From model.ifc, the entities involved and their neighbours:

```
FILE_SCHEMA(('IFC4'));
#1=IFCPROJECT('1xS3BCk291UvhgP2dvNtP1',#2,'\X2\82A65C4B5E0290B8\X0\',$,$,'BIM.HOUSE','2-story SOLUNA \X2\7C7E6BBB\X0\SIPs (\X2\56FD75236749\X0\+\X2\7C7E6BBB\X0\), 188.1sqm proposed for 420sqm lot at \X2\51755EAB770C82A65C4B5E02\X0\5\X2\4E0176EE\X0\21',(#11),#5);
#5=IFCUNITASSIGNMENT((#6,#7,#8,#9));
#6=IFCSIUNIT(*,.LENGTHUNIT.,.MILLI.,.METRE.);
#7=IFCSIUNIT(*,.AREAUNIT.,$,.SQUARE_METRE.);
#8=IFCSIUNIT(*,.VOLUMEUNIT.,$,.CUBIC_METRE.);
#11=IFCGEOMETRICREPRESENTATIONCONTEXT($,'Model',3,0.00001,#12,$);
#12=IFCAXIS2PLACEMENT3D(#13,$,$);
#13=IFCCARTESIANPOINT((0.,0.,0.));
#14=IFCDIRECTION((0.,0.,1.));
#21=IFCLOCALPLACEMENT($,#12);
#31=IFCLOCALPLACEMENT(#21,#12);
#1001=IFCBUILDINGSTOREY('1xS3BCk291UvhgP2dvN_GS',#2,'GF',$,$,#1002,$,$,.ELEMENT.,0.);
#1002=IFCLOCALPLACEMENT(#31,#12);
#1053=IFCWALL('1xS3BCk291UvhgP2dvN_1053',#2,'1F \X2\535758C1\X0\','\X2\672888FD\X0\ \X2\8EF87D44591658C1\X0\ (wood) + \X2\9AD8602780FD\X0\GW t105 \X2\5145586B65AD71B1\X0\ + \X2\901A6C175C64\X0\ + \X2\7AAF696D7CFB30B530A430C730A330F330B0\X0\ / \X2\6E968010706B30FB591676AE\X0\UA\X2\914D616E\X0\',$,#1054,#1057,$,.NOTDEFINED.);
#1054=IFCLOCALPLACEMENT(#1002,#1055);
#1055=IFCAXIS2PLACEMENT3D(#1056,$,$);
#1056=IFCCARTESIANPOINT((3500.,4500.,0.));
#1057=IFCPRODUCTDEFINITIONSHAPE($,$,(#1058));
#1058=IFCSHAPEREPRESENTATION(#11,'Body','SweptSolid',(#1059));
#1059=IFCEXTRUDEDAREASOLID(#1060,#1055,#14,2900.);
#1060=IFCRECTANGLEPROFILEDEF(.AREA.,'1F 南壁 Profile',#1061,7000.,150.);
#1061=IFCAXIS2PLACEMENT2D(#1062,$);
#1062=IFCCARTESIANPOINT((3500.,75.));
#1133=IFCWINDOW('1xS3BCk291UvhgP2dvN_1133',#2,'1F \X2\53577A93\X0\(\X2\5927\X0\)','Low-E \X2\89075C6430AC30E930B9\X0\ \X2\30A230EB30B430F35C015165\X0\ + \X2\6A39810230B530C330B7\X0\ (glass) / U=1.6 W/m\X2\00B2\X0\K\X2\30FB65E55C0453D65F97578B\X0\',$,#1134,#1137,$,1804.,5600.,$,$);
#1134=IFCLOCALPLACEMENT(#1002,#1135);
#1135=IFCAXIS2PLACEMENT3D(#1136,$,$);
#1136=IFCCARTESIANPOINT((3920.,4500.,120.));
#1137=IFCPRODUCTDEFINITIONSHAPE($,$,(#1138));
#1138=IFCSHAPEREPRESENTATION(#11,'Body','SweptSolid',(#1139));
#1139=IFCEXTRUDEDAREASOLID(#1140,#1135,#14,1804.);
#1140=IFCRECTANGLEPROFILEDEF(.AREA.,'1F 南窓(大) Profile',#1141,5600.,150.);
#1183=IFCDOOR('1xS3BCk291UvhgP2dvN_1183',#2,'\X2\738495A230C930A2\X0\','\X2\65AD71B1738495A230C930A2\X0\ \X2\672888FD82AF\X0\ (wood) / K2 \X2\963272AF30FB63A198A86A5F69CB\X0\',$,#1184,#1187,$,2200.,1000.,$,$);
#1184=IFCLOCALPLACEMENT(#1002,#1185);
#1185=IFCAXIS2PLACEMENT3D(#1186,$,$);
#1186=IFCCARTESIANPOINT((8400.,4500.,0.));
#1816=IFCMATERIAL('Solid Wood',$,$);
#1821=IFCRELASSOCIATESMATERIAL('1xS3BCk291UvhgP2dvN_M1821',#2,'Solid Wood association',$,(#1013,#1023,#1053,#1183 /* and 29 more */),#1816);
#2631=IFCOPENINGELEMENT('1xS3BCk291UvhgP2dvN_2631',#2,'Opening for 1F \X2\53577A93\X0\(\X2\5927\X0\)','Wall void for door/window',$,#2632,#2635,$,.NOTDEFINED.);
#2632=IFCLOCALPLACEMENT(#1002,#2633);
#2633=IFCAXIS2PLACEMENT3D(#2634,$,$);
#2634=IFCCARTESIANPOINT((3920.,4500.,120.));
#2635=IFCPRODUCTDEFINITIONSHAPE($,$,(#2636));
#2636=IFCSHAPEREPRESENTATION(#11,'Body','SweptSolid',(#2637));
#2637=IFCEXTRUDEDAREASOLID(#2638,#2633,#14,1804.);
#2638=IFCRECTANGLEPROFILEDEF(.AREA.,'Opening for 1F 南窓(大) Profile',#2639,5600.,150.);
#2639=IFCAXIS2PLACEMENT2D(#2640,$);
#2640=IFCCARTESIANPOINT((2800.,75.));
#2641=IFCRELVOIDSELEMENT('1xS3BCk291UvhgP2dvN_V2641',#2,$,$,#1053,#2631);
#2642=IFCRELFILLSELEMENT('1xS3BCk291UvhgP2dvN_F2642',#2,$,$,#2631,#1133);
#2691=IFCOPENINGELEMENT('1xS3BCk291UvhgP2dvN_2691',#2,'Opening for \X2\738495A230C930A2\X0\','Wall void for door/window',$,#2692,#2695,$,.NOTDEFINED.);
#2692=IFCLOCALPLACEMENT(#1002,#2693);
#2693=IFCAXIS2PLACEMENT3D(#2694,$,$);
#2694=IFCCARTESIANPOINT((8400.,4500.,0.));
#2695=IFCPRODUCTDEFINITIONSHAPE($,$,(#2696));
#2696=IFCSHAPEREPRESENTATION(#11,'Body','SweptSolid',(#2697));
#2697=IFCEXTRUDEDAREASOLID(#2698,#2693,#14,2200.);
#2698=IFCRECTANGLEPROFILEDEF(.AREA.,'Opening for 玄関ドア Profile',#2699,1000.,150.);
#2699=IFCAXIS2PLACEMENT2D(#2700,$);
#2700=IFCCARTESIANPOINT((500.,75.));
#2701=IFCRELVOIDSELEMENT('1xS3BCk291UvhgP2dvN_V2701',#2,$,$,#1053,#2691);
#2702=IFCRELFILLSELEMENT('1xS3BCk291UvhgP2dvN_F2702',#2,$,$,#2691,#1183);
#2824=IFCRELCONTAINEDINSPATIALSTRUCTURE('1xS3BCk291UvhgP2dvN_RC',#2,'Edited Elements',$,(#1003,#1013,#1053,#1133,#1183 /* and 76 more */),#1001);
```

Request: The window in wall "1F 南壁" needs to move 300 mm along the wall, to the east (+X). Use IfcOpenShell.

```python
import ifcopenshell
import ifcopenshell.api.geometry
import ifcopenshell.util.placement
import ifcopenshell.util.unit

model = ifcopenshell.open("model.ifc")
unit_scale = ifcopenshell.util.unit.calculate_unit_scale(model)

window = model.by_guid("1xS3BCk291UvhgP2dvN_1133")
opening = window.FillsVoids[0].RelatingOpeningElement
wall = opening.VoidsElements[0].RelatingBuildingElement

wall_matrix = ifcopenshell.util.placement.get_local_placement(wall.ObjectPlacement)
shift = wall_matrix[:3, 0] * 0.3 / unit_scale
before = ifcopenshell.util.placement.get_local_placement(window.ObjectPlacement)[:3, 3].copy()

# The window is not placed relative to its opening, so move both.
for product in (opening, window):
    matrix = ifcopenshell.util.placement.get_local_placement(product.ObjectPlacement)
    matrix[:3, 3] += shift
    ifcopenshell.api.geometry.edit_object_placement(model, product=product, matrix=matrix, is_si=False)

after = ifcopenshell.util.placement.get_local_placement(window.ObjectPlacement)[:3, 3]
print("window moved by", (after - before).round(3) + 0.0)

model.write("model_edited.ifc")
```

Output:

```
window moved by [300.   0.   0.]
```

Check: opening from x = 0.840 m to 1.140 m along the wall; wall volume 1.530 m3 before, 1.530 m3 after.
